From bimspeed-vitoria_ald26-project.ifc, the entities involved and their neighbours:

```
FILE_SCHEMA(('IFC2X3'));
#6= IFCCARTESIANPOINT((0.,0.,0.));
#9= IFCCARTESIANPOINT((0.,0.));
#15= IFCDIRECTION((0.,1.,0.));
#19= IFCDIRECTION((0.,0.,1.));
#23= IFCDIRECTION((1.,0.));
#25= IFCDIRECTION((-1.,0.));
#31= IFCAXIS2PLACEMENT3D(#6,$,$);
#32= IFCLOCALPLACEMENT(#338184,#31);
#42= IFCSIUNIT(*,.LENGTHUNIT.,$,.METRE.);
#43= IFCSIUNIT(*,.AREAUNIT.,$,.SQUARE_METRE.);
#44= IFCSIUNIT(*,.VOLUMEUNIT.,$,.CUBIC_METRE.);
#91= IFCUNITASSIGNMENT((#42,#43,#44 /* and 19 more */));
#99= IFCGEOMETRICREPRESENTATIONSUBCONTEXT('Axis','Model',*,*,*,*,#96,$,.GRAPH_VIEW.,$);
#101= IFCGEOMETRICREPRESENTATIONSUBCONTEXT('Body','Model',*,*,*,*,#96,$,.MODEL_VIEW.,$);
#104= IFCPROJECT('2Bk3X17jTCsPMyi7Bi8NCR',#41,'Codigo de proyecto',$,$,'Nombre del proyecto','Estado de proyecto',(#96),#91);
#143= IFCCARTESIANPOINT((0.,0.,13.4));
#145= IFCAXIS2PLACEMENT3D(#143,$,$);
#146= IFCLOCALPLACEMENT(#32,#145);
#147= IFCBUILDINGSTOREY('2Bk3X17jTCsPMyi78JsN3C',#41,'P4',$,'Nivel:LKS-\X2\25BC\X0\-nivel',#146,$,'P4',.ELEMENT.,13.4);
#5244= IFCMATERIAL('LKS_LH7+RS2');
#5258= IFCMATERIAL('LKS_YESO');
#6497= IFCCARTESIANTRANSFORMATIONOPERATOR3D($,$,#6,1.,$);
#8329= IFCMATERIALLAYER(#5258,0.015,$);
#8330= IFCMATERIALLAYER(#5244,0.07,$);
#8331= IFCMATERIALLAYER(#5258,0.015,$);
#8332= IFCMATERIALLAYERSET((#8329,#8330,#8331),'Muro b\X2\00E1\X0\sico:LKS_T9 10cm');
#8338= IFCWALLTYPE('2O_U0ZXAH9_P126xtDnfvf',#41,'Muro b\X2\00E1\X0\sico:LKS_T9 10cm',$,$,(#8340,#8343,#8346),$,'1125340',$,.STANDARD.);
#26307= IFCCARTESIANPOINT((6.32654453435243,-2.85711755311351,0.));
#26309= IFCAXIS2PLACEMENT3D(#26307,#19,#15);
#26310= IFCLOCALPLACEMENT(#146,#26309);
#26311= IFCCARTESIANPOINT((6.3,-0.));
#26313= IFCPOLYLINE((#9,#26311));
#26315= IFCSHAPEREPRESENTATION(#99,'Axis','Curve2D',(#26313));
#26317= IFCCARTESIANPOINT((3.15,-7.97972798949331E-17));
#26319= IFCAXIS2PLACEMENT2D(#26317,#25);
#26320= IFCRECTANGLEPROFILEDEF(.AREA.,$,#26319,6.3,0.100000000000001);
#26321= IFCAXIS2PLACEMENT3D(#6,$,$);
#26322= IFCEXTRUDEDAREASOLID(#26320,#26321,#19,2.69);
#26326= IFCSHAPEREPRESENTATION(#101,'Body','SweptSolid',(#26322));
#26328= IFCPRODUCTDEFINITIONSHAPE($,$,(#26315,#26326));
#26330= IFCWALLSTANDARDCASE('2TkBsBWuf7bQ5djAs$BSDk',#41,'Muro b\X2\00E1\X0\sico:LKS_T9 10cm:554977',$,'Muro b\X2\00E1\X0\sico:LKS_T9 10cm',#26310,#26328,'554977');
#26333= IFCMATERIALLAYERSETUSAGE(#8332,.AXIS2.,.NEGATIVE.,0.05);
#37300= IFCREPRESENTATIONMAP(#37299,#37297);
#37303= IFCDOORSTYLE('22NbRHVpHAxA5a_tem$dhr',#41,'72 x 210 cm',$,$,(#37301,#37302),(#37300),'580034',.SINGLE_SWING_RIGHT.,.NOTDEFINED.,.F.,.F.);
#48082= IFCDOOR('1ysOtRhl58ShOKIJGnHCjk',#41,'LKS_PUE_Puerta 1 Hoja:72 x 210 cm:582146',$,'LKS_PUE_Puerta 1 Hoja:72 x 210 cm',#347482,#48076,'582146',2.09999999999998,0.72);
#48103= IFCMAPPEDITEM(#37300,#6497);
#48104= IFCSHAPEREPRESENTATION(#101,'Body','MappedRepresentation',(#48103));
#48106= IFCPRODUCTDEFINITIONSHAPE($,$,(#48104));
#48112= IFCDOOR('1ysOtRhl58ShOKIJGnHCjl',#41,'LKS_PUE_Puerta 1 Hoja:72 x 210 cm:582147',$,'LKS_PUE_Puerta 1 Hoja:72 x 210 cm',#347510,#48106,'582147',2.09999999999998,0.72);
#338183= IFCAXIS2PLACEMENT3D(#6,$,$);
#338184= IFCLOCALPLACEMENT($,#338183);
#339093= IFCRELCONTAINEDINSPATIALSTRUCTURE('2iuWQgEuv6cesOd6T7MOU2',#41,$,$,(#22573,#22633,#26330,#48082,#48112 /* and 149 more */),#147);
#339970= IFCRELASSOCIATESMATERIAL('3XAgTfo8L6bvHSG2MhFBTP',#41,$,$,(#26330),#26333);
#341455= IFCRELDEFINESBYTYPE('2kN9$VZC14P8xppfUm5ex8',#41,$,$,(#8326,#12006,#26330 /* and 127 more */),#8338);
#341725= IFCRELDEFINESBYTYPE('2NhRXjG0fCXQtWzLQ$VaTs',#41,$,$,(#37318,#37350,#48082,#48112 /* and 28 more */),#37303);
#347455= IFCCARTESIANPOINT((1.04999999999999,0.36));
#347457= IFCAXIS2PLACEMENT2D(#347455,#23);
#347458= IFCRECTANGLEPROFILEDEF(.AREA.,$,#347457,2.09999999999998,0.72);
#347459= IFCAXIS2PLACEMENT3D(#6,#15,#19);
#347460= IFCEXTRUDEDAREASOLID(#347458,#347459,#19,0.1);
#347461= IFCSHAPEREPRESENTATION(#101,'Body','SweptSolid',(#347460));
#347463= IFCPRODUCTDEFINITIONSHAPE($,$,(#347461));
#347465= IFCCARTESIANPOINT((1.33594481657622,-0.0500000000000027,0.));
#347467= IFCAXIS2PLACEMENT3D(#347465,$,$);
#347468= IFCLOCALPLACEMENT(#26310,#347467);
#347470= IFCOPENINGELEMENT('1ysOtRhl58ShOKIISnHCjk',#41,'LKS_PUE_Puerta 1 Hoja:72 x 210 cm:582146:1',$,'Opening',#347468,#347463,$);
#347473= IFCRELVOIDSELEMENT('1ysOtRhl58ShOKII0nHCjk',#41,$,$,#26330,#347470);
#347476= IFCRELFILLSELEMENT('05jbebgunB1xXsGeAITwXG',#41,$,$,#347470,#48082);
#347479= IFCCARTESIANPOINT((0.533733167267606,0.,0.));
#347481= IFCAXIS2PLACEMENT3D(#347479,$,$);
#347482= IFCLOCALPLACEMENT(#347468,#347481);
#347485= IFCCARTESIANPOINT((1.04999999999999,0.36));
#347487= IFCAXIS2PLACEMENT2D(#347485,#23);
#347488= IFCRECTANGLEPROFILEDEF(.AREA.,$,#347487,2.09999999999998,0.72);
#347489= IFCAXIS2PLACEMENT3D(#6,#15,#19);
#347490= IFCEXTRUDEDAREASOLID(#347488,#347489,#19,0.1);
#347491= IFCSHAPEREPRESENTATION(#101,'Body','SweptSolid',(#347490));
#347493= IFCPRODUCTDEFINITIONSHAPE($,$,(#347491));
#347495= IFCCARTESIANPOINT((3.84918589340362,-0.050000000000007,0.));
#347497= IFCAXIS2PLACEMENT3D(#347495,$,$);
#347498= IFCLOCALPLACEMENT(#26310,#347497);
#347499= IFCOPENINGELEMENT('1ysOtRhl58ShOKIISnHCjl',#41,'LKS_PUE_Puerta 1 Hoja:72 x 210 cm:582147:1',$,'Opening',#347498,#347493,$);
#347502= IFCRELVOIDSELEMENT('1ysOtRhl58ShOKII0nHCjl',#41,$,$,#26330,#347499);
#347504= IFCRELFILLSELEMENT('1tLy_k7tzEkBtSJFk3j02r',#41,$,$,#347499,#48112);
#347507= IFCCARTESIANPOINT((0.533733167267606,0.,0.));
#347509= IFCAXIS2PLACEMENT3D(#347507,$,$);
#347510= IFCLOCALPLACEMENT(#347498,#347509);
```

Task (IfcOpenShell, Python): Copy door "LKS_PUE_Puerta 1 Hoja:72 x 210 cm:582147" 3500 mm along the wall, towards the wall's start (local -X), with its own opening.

```python
import ifcopenshell
import ifcopenshell.api.feature
import ifcopenshell.api.geometry
import ifcopenshell.api.root
import ifcopenshell.geom
import ifcopenshell.util.element
import ifcopenshell.util.placement
import ifcopenshell.util.shape

model = ifcopenshell.open("bimspeed-vitoria_ald26-project.ifc")
settings = ifcopenshell.geom.settings()


def volume(element):
    """Net volume in cubic metres, openings subtracted."""
    shape = ifcopenshell.geom.create_shape(settings, element)
    return ifcopenshell.util.shape.get_volume(shape.geometry)


def reuse_history(source, copy):
    """copy_class also copies each property set's owner history, people and application; keep the originals."""
    for rel in copy.IsDefinedBy:
        if rel.is_a("IfcRelDefinesByProperties") and (history := rel.RelatingPropertyDefinition.OwnerHistory):
            rel.RelatingPropertyDefinition.OwnerHistory = source.OwnerHistory
            ifcopenshell.util.element.remove_deep2(model, history)


door = model.by_id(48112)
opening = door.FillsVoids[0].RelatingOpeningElement
wall = opening.VoidsElements[0].RelatingBuildingElement
before = volume(wall)
shift = ifcopenshell.util.placement.get_local_placement(wall.ObjectPlacement)[:3, 0] * -3.5

# copy_class copies the void relationship, type, container and properties, but no geometry.
new_opening = ifcopenshell.api.root.copy_class(model, product=opening)
new_opening.Representation = ifcopenshell.util.element.copy_deep(
    model, opening.Representation, exclude=["IfcGeometricRepresentationContext", "IfcRepresentationMap"]
)
new_opening.Name = "LKS_PUE_Puerta 1 Hoja:72 x 210 cm"
new_door = ifcopenshell.api.root.copy_class(model, product=door)
new_door.Representation = ifcopenshell.util.element.copy_deep(
    model, door.Representation, exclude=["IfcGeometricRepresentationContext", "IfcRepresentationMap"]
)
new_door.Name = "LKS_PUE_Puerta 1 Hoja:72 x 210 cm"
new_door.Tag = None
reuse_history(door, new_door)
fills = ifcopenshell.api.feature.add_filling(model, opening=new_opening, element=new_door)
fills.OwnerHistory = new_door.OwnerHistory  # required in IFC2X3

for old, new in ((opening, new_opening), (door, new_door)):
    matrix = ifcopenshell.util.placement.get_local_placement(old.ObjectPlacement)
    matrix[:3, 3] += shift
    ifcopenshell.api.geometry.edit_object_placement(model, product=new, matrix=matrix, is_si=False)

after = volume(wall)

print(f"wall volume {before:.3f} -> {after:.3f} m3")

model.write("bimspeed-vitoria_ald26-project_updated.ifc")
```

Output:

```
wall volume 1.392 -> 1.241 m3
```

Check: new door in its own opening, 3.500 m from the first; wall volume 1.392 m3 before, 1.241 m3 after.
